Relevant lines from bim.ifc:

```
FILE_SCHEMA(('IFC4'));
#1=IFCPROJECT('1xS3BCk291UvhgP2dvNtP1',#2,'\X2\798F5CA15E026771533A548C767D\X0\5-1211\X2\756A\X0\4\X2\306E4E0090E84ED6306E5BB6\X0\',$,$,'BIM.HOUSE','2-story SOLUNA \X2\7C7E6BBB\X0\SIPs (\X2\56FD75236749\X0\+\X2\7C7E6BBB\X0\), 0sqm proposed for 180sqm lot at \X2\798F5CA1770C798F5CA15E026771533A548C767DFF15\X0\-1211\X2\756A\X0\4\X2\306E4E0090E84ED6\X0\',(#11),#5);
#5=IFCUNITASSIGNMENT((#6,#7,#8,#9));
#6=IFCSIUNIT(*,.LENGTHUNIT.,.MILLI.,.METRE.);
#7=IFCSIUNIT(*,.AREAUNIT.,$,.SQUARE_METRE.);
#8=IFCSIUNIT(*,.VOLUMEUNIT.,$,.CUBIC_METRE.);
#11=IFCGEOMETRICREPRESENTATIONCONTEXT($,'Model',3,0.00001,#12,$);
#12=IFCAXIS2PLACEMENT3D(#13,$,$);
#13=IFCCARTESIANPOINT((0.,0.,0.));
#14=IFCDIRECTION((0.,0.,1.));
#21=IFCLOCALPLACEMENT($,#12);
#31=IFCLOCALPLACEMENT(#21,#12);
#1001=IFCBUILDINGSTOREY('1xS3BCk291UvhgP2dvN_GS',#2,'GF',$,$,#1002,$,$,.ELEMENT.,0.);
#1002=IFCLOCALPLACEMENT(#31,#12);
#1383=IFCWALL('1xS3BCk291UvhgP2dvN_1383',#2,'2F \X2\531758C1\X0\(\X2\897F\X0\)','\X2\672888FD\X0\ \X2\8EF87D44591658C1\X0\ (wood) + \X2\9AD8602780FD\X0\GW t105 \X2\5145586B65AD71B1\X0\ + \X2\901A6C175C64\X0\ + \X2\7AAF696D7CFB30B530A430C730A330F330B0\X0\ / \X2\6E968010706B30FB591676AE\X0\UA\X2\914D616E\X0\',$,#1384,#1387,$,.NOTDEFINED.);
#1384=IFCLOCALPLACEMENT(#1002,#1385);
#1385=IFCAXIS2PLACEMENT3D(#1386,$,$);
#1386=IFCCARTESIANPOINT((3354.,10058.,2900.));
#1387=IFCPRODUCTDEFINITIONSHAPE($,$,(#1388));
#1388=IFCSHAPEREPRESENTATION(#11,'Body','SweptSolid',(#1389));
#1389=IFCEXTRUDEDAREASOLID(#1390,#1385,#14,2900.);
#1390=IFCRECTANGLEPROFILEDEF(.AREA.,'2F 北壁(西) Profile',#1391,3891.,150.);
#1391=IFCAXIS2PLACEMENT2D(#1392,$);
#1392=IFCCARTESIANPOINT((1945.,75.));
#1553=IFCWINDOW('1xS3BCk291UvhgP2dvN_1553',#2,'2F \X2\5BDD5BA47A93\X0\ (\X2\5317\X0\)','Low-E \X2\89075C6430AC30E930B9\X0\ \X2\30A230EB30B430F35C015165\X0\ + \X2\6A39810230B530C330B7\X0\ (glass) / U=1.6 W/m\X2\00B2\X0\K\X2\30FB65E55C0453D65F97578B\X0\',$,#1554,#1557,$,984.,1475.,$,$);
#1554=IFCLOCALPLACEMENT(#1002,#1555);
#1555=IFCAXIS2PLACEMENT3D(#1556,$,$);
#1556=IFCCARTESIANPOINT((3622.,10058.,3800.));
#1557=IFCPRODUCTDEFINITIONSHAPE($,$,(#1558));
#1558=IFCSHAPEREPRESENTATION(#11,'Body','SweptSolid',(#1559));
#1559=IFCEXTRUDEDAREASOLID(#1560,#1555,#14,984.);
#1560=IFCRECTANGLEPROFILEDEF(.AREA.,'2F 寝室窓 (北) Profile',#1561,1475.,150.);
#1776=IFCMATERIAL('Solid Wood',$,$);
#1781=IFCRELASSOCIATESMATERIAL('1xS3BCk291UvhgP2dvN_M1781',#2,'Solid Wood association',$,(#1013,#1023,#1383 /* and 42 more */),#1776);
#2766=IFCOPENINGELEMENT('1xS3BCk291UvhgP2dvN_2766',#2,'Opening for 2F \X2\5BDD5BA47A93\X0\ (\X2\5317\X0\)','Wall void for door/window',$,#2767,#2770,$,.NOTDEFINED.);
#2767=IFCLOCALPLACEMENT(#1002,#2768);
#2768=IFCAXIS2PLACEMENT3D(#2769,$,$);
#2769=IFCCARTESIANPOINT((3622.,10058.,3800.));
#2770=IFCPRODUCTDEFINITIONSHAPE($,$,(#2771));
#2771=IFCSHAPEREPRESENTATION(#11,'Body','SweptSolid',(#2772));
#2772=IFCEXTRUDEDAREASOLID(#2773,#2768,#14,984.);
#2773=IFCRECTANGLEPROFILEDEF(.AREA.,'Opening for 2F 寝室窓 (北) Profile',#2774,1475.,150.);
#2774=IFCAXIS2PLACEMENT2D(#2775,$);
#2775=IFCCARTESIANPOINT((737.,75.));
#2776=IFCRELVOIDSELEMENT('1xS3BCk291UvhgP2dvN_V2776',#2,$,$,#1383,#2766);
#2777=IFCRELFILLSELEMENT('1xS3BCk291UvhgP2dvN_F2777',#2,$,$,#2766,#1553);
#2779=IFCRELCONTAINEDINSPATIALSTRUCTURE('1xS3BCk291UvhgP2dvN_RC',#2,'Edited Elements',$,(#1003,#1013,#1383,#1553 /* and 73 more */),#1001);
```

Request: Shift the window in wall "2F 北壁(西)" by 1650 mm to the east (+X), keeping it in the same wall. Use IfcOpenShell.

```python
import ifcopenshell
import ifcopenshell.api.geometry
import ifcopenshell.util.placement
import ifcopenshell.util.unit

model = ifcopenshell.open("bim.ifc")
unit_scale = ifcopenshell.util.unit.calculate_unit_scale(model)

window = model.by_guid("1xS3BCk291UvhgP2dvN_1553")
opening = window.FillsVoids[0].RelatingOpeningElement
wall = opening.VoidsElements[0].RelatingBuildingElement

wall_matrix = ifcopenshell.util.placement.get_local_placement(wall.ObjectPlacement)
shift = wall_matrix[:3, 0] * 1.65 / unit_scale
before = ifcopenshell.util.placement.get_local_placement(window.ObjectPlacement)[:3, 3].copy()

# The window is not placed relative to its opening, so move both.
for product in (opening, window):
    matrix = ifcopenshell.util.placement.get_local_placement(product.ObjectPlacement)
    matrix[:3, 3] += shift
    ifcopenshell.api.geometry.edit_object_placement(model, product=product, matrix=matrix, is_si=False)

after = ifcopenshell.util.placement.get_local_placement(window.ObjectPlacement)[:3, 3]
print("window moved by", (after - before).round(3) + 0.0)

model.write("bim_v2.ifc")
```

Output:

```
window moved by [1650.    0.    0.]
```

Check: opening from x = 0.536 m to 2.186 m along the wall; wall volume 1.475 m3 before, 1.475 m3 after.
